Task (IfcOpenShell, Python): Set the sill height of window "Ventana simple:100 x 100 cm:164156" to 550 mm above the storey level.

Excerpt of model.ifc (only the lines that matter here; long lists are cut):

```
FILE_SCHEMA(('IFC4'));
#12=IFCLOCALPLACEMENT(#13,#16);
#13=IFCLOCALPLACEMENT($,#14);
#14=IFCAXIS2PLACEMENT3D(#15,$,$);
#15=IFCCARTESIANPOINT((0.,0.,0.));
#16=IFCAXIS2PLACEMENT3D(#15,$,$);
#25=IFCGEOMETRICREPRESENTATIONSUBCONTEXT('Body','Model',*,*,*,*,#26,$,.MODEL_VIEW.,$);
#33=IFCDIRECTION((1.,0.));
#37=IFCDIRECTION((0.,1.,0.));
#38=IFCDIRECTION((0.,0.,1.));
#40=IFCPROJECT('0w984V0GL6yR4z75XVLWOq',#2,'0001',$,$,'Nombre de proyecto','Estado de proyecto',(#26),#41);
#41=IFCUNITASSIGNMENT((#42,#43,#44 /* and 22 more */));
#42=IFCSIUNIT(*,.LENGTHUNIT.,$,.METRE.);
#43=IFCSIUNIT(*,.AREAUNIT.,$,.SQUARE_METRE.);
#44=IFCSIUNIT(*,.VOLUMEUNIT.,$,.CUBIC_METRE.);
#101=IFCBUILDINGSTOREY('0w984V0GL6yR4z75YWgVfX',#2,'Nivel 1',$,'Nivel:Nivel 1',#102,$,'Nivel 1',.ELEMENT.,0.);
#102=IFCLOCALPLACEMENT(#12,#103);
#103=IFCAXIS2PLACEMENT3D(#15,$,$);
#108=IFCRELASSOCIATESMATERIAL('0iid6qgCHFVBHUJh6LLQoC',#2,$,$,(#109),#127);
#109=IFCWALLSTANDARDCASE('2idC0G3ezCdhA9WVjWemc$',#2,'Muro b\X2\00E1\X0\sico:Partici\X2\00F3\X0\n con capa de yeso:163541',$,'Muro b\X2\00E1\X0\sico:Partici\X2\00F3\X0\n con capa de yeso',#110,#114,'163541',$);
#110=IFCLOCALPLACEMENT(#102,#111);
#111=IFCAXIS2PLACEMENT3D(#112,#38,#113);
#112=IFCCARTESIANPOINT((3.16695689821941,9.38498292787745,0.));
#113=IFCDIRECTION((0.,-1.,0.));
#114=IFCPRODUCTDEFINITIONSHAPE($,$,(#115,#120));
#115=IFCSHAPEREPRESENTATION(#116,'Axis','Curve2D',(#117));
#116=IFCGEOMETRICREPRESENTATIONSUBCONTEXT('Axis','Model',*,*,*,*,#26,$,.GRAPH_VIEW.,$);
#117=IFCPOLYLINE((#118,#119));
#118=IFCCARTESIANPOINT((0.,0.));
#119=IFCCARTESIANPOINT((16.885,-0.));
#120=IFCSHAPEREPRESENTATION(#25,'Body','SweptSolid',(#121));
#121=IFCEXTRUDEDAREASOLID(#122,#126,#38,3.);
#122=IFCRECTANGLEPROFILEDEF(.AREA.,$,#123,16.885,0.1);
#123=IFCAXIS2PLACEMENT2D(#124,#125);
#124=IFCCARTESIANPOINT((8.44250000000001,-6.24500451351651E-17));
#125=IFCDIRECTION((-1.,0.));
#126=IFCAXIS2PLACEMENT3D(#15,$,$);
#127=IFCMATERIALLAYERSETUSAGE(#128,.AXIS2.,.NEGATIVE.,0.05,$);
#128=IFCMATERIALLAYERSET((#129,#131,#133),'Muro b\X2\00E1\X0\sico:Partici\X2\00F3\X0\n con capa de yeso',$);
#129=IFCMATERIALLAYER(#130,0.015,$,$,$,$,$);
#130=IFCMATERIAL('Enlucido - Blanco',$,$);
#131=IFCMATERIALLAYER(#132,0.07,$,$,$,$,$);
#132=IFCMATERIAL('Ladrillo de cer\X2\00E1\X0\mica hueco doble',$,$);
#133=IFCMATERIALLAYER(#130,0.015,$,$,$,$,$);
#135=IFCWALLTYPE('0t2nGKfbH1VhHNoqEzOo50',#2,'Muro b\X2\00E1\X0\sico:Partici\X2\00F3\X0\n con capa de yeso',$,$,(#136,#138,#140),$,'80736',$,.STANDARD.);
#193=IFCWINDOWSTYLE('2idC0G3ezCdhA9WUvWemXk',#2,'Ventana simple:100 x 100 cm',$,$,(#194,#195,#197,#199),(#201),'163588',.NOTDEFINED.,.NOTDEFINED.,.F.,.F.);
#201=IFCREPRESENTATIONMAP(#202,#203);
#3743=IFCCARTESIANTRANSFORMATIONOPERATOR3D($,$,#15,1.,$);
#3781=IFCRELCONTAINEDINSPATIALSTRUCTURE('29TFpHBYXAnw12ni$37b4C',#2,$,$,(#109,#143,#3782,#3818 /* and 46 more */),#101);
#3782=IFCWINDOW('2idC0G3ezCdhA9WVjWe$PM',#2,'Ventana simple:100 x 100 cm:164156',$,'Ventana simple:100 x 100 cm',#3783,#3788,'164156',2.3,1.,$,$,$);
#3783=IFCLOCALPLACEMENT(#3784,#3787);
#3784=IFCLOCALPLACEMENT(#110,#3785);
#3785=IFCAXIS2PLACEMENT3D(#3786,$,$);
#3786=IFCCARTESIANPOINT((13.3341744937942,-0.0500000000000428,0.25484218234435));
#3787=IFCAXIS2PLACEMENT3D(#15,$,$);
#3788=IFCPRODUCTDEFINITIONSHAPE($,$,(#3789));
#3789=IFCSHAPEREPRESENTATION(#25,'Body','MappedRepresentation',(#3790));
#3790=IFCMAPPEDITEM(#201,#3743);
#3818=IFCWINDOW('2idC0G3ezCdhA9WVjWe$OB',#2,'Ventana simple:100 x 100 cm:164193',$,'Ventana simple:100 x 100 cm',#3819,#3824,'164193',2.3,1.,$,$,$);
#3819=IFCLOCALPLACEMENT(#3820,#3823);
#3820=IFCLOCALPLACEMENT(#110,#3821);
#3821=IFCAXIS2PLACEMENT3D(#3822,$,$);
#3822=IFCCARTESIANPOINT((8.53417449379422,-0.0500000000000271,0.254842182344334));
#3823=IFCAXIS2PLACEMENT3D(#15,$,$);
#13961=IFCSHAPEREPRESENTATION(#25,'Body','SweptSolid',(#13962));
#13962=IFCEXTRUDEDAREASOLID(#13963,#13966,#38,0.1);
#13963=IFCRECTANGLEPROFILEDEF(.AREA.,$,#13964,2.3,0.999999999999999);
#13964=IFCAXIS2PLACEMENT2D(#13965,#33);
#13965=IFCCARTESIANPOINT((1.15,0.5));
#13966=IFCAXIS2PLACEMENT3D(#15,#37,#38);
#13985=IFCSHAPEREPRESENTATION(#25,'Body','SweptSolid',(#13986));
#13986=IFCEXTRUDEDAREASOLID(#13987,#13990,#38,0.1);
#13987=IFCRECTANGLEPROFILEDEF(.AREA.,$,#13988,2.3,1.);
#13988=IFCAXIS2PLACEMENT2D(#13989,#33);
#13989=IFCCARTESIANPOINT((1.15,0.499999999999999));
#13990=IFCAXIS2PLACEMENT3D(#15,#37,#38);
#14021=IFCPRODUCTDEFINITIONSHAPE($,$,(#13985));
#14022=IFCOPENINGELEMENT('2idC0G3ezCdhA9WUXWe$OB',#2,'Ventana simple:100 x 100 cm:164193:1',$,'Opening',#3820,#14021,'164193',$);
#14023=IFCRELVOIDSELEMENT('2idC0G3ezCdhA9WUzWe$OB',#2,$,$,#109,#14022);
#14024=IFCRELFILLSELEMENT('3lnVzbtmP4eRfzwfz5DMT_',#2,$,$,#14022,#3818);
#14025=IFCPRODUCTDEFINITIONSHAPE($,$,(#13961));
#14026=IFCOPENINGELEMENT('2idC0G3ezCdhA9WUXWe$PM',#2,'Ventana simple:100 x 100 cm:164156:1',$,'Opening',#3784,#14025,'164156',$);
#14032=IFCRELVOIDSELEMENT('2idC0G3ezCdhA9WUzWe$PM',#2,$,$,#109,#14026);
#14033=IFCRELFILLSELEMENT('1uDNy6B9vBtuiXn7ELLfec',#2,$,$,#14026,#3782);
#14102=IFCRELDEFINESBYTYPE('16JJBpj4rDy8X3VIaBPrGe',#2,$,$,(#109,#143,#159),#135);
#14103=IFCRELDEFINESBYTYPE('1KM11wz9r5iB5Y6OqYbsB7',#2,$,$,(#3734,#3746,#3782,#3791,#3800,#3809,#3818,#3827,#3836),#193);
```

```python
import numpy as np
import ifcopenshell
import ifcopenshell.api.geometry
import ifcopenshell.geom
import ifcopenshell.util.element
import ifcopenshell.util.placement
import ifcopenshell.util.shape
import ifcopenshell.util.unit

model = ifcopenshell.open("model.ifc")
unit_scale = ifcopenshell.util.unit.calculate_unit_scale(model)

window = model.by_guid("2idC0G3ezCdhA9WVjWe$PM")
opening = window.FillsVoids[0].RelatingOpeningElement
storey = ifcopenshell.util.element.get_container(window, ifc_class="IfcBuildingStorey")
level = ifcopenshell.util.placement.get_local_placement(storey.ObjectPlacement)[2, 3]

# The opening's origin need not be at the sill, so measure its lowest point.
shape = ifcopenshell.geom.create_shape(ifcopenshell.geom.settings(), opening)
bottom = ifcopenshell.util.shape.get_shape_bottom_elevation(shape, shape.geometry) / unit_scale
dz = level + 0.55 / unit_scale - bottom

shift = np.array([0.0, 0.0, dz])
# The window is placed relative to its opening, so it follows when the opening moves.
matrix = ifcopenshell.util.placement.get_local_placement(opening.ObjectPlacement)
matrix[:3, 3] += shift
ifcopenshell.api.geometry.edit_object_placement(
    model, product=opening, matrix=matrix, is_si=False, should_transform_children=True
)

print(f"moved by {dz * unit_scale:+.3f} m")

model.write("model_rev.ifc")
```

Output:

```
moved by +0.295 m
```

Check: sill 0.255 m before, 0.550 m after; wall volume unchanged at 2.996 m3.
